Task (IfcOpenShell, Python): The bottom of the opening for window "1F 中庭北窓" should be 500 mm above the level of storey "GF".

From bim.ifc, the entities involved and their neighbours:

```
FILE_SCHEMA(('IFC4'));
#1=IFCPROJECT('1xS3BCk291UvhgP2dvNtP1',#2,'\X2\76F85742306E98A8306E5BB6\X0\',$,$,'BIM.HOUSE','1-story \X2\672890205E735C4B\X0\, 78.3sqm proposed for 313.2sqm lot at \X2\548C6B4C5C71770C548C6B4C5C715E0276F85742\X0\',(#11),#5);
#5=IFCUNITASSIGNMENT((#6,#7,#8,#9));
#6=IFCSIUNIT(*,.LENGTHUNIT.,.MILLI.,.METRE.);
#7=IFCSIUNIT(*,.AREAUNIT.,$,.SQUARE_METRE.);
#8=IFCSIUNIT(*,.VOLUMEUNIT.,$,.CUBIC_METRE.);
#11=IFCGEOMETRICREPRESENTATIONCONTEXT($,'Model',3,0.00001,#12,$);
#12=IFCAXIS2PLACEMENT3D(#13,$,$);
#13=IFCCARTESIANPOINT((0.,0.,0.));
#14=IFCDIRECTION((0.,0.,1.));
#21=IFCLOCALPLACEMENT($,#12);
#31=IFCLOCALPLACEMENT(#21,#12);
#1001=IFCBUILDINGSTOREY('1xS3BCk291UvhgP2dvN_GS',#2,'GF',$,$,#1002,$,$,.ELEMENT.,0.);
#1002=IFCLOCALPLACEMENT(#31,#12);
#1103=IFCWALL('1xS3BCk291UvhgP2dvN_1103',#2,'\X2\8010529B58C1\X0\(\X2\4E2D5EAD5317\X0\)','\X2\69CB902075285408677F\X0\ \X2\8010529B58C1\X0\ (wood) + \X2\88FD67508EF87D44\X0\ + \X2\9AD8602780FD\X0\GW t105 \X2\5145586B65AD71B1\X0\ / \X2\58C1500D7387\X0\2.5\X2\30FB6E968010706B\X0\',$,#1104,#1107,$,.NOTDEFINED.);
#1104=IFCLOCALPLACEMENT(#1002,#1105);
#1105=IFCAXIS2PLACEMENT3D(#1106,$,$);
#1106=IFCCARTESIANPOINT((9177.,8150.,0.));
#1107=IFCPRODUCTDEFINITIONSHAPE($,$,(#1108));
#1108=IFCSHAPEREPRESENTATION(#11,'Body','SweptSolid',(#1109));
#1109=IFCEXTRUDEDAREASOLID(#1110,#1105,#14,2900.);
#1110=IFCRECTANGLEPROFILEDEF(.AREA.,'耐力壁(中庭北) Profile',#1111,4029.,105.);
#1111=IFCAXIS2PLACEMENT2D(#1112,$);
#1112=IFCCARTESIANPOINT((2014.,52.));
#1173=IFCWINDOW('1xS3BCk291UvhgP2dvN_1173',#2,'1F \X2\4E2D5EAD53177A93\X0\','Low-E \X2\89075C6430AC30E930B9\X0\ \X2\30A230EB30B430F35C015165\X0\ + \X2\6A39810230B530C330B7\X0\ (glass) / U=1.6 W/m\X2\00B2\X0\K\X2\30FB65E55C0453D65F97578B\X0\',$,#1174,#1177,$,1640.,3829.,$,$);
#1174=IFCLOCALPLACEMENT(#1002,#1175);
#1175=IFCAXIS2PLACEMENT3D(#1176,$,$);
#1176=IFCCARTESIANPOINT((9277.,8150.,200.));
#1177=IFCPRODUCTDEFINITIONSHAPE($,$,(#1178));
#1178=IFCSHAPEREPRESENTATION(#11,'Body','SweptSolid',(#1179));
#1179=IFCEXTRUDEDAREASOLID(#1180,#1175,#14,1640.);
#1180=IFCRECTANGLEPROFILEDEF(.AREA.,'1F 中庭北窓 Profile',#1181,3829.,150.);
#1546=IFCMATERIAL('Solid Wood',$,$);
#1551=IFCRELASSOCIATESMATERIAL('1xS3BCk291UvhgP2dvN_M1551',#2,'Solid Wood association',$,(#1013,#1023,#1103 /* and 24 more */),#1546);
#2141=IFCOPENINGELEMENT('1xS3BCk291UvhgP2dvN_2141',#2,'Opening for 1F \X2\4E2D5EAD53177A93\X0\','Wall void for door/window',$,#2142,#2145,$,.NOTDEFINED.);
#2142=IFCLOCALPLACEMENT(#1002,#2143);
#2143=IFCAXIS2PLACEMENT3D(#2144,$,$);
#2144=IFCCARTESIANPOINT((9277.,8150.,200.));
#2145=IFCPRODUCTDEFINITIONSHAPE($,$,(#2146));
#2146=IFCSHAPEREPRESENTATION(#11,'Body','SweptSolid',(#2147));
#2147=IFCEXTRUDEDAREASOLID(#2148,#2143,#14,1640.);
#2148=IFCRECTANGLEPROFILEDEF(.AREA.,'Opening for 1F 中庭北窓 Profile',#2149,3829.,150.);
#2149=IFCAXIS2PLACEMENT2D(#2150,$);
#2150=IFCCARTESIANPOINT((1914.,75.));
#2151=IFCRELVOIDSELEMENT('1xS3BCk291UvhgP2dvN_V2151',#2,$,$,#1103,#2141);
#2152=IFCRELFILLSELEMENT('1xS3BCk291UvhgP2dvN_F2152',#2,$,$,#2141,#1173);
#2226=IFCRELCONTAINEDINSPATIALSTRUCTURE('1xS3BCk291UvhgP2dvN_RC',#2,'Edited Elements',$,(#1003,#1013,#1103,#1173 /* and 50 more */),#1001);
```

```python
import numpy as np
import ifcopenshell
import ifcopenshell.api.geometry
import ifcopenshell.geom
import ifcopenshell.util.element
import ifcopenshell.util.placement
import ifcopenshell.util.shape
import ifcopenshell.util.unit

model = ifcopenshell.open("bim.ifc")
unit_scale = ifcopenshell.util.unit.calculate_unit_scale(model)

window = model.by_guid("1xS3BCk291UvhgP2dvN_1173")
opening = window.FillsVoids[0].RelatingOpeningElement
storey = ifcopenshell.util.element.get_container(window, ifc_class="IfcBuildingStorey")
level = ifcopenshell.util.placement.get_local_placement(storey.ObjectPlacement)[2, 3]

# The opening's origin need not be at the sill, so measure its lowest point.
shape = ifcopenshell.geom.create_shape(ifcopenshell.geom.settings(), opening)
bottom = ifcopenshell.util.shape.get_shape_bottom_elevation(shape, shape.geometry) / unit_scale
dz = level + 500.0 - bottom

shift = np.array([0.0, 0.0, dz])
# The window is not placed relative to its opening, so move both.
for product in (opening, window):
    matrix = ifcopenshell.util.placement.get_local_placement(product.ObjectPlacement)
    matrix[:3, 3] += shift
    ifcopenshell.api.geometry.edit_object_placement(model, product=product, matrix=matrix, is_si=False)

print(f"moved by {dz * unit_scale:+.3f} m")

model.write("bim_updated.ifc")
```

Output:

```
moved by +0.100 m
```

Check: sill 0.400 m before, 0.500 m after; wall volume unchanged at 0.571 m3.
